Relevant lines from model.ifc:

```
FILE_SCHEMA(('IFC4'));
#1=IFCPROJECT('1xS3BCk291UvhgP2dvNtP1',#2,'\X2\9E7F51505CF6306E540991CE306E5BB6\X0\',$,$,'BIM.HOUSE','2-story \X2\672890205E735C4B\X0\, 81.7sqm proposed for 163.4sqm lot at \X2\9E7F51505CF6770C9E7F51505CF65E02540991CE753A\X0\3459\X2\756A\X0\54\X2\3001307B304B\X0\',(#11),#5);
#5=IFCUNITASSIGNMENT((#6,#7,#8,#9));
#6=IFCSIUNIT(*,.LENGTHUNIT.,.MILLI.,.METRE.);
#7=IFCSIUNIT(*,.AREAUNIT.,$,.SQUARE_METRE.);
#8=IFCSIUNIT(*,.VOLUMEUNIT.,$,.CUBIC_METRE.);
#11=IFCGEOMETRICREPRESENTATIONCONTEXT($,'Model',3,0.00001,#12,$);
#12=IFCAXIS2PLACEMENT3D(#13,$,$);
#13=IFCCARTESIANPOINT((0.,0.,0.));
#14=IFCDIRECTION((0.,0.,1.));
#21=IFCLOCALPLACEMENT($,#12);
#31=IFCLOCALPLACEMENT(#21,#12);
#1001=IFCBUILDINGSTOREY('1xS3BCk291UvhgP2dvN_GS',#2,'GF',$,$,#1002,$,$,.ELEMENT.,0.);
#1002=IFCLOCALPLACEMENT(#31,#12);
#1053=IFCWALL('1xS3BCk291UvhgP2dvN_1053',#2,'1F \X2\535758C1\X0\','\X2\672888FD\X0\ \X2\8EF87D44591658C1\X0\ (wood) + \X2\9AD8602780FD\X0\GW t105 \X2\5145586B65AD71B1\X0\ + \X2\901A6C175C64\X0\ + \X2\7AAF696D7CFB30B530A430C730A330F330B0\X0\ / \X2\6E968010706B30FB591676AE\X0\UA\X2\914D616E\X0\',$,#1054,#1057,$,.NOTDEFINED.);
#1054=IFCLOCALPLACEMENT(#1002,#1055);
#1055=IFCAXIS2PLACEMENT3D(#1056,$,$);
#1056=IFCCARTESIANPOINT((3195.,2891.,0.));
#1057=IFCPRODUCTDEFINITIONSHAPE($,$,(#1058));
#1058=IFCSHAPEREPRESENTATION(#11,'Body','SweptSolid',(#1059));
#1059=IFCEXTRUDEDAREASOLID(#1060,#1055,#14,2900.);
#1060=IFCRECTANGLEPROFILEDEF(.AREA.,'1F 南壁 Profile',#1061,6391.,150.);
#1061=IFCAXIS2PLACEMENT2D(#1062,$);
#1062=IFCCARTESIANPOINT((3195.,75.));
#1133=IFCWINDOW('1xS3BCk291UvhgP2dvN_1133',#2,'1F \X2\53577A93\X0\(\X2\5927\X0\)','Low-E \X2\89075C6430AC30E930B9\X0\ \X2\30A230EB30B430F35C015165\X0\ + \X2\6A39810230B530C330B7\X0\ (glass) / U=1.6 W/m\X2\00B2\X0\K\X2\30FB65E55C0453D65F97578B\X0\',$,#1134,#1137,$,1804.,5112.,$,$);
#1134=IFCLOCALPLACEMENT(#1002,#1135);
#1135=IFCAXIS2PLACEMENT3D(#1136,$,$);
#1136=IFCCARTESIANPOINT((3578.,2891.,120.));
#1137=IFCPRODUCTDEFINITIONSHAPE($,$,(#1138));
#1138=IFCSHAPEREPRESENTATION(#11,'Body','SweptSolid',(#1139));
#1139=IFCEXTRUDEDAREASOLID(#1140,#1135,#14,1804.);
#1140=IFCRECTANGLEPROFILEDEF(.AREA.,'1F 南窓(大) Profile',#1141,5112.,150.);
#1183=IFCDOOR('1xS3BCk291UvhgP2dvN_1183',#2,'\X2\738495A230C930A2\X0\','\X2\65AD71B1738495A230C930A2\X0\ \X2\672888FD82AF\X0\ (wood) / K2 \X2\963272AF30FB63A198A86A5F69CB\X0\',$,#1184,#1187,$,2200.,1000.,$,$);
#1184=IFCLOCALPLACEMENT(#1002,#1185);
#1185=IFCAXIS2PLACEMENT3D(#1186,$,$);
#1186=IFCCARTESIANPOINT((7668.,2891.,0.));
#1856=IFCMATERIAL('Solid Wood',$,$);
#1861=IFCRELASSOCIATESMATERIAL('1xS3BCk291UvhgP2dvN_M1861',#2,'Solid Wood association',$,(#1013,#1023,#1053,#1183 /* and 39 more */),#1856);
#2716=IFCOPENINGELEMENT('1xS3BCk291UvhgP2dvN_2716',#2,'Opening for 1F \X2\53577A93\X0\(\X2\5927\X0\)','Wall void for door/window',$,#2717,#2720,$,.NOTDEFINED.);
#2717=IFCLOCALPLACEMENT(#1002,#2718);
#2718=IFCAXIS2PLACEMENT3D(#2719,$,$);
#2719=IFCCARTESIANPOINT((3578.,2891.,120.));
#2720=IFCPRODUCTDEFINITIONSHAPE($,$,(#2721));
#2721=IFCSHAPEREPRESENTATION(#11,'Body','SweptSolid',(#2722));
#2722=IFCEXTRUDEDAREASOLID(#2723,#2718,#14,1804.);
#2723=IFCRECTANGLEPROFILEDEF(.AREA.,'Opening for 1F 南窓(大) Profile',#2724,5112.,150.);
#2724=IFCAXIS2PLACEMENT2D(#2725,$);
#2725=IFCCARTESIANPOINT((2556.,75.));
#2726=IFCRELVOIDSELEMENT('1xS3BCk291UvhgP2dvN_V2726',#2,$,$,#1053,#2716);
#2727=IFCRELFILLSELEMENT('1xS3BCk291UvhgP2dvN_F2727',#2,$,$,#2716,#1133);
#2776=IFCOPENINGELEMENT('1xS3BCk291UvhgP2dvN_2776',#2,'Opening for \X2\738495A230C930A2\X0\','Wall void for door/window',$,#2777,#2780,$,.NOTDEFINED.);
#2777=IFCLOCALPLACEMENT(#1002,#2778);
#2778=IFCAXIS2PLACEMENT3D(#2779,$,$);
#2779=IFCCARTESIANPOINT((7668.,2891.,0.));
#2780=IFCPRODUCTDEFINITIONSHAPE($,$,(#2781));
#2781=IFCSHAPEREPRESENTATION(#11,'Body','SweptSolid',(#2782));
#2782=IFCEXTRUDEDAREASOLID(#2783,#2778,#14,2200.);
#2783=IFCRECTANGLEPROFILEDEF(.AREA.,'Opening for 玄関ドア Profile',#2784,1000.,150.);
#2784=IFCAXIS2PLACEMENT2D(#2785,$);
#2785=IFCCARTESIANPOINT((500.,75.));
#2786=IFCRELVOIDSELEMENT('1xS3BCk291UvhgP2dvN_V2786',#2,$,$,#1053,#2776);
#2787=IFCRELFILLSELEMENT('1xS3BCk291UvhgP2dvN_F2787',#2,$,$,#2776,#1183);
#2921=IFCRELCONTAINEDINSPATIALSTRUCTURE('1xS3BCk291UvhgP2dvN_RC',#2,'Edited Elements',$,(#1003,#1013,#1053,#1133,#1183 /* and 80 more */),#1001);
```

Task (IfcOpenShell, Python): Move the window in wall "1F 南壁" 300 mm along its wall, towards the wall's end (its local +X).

```python
import ifcopenshell
import ifcopenshell.api.geometry
import ifcopenshell.util.placement

model = ifcopenshell.open("model.ifc")

window = model.by_guid("1xS3BCk291UvhgP2dvN_1133")
opening = window.FillsVoids[0].RelatingOpeningElement
wall = opening.VoidsElements[0].RelatingBuildingElement

wall_matrix = ifcopenshell.util.placement.get_local_placement(wall.ObjectPlacement)
shift = wall_matrix[:3, 0] * 300.0
before = ifcopenshell.util.placement.get_local_placement(window.ObjectPlacement)[:3, 3].copy()

# The window is not placed relative to its opening, so move both.
for product in (opening, window):
    matrix = ifcopenshell.util.placement.get_local_placement(product.ObjectPlacement)
    matrix[:3, 3] += shift
    ifcopenshell.api.geometry.edit_object_placement(model, product=product, matrix=matrix, is_si=False)

after = ifcopenshell.util.placement.get_local_placement(window.ObjectPlacement)[:3, 3]
print("window moved by", (after - before).round(3) + 0.0)

model.write("model_rev.ifc")
```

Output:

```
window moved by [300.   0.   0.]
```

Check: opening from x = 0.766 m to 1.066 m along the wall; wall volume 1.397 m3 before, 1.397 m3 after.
